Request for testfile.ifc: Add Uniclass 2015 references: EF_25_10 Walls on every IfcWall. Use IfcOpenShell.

First a look at what the model holds.

```python
import ifcopenshell

model = ifcopenshell.open("testfile.ifc")
print(model.schema)
print("classifications:", [c.Name for c in model.by_type("IfcClassification")])
for ifc_class in ("IfcDoor", "IfcRoof", "IfcStair", "IfcWall", "IfcWindow"):
    print(ifc_class, len(model.by_type(ifc_class)))
```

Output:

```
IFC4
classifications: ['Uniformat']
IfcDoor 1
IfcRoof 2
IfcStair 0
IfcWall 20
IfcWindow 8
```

```python
import ifcopenshell
import ifcopenshell.api.classification

model = ifcopenshell.open("testfile.ifc")

system = ifcopenshell.api.classification.add_classification(model, classification="Uniclass 2015")

codes = {
    "IfcWall": ("EF_25_10", "Walls"),
}
for ifc_class, (code, name) in codes.items():
    products = model.by_type(ifc_class)
    ifcopenshell.api.classification.add_reference(
        model, products=products, classification=system, identification=code, name=name
    )
    print(code, len(products))

model.write("testfile_edited.ifc")
```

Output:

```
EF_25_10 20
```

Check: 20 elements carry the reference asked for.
